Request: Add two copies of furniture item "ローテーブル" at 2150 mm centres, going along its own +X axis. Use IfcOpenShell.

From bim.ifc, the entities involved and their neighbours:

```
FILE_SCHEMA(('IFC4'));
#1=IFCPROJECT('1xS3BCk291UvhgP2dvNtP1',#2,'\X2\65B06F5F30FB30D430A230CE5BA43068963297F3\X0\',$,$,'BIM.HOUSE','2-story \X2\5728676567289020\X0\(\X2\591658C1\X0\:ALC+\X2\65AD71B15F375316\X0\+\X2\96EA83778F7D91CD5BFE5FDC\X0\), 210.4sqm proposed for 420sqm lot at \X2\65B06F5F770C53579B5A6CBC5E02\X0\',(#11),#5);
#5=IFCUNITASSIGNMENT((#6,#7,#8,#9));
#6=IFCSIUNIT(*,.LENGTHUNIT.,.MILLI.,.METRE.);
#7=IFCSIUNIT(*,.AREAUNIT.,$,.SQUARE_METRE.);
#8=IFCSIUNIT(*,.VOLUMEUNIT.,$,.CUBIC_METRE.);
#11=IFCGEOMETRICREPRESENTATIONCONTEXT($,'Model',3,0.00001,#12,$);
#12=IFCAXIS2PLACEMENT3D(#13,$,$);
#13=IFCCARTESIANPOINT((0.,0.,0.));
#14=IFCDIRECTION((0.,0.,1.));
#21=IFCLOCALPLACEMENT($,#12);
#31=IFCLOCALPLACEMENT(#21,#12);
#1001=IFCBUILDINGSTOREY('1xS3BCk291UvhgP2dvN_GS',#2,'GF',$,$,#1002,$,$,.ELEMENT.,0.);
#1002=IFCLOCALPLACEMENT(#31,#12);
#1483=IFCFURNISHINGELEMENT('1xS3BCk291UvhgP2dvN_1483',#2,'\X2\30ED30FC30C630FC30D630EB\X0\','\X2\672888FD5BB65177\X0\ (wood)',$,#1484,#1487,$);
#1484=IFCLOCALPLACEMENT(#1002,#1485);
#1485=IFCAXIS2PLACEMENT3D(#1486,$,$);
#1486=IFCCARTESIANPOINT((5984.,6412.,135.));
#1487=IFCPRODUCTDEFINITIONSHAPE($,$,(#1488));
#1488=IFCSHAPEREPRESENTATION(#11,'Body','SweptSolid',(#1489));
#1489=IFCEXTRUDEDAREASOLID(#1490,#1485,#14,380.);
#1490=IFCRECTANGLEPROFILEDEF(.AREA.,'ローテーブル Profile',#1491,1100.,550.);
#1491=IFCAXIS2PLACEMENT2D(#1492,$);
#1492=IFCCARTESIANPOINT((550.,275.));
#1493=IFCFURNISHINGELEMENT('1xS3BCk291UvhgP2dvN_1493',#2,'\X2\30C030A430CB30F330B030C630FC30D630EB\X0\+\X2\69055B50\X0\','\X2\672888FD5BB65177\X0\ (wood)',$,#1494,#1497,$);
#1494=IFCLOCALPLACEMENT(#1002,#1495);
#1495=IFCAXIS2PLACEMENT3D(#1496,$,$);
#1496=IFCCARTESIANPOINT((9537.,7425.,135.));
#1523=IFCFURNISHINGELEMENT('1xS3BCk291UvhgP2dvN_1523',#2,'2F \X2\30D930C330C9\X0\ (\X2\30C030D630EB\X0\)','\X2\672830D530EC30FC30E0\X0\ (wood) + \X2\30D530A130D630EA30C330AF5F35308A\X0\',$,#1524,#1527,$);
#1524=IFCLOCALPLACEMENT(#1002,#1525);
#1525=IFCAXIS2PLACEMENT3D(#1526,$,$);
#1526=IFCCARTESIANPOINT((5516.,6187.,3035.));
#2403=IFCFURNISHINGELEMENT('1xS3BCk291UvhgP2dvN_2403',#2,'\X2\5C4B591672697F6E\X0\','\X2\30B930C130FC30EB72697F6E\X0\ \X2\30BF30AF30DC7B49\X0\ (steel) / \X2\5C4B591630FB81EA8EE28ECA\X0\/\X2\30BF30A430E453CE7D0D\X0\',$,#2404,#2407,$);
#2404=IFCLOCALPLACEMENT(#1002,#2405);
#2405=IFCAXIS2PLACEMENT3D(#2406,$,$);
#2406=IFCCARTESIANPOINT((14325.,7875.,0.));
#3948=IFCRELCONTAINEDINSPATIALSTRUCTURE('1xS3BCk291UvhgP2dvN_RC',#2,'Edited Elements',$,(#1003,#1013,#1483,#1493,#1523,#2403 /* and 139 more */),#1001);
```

```python
import ifcopenshell
import ifcopenshell.api.geometry
import ifcopenshell.api.root
import ifcopenshell.util.element
import ifcopenshell.util.placement
import ifcopenshell.util.unit

model = ifcopenshell.open("bim.ifc")
unit_scale = ifcopenshell.util.unit.calculate_unit_scale(model)


def reuse_history(source, copy):
    """copy_class also copies each property set's owner history, people and application; keep the originals."""
    for rel in copy.IsDefinedBy:
        if rel.is_a("IfcRelDefinesByProperties") and (history := rel.RelatingPropertyDefinition.OwnerHistory):
            rel.RelatingPropertyDefinition.OwnerHistory = source.OwnerHistory
            ifcopenshell.util.element.remove_deep2(model, history)


source = model.by_id(1483)
base = ifcopenshell.util.placement.get_local_placement(source.ObjectPlacement)
step = base[:3, 0] * 2.15 / unit_scale

for i in range(1, 3):
    copy = ifcopenshell.api.root.copy_class(model, product=source)
    copy.Representation = ifcopenshell.util.element.copy_deep(
        model, source.Representation, exclude=["IfcGeometricRepresentationContext", "IfcRepresentationMap"]
    )
    reuse_history(source, copy)
    matrix = base.copy()
    matrix[:3, 3] += i * step
    print("added at", matrix[:3, 3].round(3) + 0.0)
    ifcopenshell.api.geometry.edit_object_placement(model, product=copy, matrix=matrix, is_si=False)

model.write("bim_v2.ifc")
```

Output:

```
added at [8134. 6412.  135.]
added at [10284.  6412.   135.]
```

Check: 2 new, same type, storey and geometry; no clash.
